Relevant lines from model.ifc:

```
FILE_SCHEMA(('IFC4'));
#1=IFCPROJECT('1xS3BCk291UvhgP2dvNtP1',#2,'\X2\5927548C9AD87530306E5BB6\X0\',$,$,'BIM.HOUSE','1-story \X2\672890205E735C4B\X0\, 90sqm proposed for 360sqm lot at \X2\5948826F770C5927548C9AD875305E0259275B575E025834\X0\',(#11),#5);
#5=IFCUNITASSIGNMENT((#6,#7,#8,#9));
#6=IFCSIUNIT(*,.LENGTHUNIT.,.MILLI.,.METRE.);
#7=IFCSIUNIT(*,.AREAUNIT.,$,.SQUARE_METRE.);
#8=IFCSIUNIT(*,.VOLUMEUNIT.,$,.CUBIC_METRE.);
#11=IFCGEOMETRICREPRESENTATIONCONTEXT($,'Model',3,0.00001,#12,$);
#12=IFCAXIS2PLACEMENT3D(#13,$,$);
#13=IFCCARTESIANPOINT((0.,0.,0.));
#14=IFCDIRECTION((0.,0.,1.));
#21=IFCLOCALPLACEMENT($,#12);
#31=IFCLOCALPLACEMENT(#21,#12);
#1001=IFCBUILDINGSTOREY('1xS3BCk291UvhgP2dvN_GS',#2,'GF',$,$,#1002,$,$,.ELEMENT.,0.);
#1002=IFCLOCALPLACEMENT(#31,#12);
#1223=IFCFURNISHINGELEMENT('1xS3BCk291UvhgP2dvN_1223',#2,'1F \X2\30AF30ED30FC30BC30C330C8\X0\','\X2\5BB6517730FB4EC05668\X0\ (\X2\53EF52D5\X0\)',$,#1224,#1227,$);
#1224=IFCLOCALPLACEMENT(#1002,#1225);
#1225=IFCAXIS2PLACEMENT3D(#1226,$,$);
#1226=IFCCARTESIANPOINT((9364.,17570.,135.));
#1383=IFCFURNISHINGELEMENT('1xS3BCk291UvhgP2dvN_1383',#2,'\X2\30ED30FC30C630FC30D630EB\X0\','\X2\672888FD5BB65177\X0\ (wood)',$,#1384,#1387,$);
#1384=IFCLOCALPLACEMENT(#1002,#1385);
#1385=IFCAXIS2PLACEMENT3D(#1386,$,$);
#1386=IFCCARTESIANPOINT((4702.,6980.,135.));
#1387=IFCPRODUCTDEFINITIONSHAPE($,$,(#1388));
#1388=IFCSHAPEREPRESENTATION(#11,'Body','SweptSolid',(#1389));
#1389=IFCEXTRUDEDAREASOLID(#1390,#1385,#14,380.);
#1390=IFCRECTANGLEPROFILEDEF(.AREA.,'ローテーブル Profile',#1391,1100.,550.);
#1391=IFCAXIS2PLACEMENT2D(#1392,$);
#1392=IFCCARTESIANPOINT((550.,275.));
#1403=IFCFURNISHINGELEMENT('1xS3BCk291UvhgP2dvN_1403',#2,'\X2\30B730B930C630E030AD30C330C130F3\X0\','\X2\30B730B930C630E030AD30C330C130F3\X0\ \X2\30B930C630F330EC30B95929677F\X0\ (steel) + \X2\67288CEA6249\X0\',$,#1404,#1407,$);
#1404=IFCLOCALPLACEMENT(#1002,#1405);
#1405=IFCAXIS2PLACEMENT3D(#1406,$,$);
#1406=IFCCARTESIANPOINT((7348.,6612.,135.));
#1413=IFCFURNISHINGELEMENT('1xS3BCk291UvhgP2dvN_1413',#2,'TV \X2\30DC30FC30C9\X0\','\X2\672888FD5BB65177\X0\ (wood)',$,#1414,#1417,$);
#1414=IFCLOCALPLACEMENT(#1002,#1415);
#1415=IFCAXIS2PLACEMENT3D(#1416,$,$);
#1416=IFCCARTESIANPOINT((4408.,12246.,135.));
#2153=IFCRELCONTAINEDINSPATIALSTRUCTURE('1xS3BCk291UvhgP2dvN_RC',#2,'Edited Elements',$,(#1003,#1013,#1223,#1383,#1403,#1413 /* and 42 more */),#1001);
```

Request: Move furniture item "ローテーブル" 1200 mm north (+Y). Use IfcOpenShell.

```python
import ifcopenshell
import ifcopenshell.api.geometry
import ifcopenshell.util.placement

model = ifcopenshell.open("model.ifc")

item = model.by_guid("1xS3BCk291UvhgP2dvN_1383")
matrix = ifcopenshell.util.placement.get_local_placement(item.ObjectPlacement)
matrix[1, 3] += 1200.0
ifcopenshell.api.geometry.edit_object_placement(model, product=item, matrix=matrix, is_si=False)

print(ifcopenshell.util.placement.get_local_placement(item.ObjectPlacement).round(3) + 0.0)

model.write("model_updated.ifc")
```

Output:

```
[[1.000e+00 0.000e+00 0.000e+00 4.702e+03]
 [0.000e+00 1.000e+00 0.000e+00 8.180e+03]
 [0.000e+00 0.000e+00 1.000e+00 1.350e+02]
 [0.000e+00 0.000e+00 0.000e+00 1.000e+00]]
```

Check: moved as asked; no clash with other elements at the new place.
